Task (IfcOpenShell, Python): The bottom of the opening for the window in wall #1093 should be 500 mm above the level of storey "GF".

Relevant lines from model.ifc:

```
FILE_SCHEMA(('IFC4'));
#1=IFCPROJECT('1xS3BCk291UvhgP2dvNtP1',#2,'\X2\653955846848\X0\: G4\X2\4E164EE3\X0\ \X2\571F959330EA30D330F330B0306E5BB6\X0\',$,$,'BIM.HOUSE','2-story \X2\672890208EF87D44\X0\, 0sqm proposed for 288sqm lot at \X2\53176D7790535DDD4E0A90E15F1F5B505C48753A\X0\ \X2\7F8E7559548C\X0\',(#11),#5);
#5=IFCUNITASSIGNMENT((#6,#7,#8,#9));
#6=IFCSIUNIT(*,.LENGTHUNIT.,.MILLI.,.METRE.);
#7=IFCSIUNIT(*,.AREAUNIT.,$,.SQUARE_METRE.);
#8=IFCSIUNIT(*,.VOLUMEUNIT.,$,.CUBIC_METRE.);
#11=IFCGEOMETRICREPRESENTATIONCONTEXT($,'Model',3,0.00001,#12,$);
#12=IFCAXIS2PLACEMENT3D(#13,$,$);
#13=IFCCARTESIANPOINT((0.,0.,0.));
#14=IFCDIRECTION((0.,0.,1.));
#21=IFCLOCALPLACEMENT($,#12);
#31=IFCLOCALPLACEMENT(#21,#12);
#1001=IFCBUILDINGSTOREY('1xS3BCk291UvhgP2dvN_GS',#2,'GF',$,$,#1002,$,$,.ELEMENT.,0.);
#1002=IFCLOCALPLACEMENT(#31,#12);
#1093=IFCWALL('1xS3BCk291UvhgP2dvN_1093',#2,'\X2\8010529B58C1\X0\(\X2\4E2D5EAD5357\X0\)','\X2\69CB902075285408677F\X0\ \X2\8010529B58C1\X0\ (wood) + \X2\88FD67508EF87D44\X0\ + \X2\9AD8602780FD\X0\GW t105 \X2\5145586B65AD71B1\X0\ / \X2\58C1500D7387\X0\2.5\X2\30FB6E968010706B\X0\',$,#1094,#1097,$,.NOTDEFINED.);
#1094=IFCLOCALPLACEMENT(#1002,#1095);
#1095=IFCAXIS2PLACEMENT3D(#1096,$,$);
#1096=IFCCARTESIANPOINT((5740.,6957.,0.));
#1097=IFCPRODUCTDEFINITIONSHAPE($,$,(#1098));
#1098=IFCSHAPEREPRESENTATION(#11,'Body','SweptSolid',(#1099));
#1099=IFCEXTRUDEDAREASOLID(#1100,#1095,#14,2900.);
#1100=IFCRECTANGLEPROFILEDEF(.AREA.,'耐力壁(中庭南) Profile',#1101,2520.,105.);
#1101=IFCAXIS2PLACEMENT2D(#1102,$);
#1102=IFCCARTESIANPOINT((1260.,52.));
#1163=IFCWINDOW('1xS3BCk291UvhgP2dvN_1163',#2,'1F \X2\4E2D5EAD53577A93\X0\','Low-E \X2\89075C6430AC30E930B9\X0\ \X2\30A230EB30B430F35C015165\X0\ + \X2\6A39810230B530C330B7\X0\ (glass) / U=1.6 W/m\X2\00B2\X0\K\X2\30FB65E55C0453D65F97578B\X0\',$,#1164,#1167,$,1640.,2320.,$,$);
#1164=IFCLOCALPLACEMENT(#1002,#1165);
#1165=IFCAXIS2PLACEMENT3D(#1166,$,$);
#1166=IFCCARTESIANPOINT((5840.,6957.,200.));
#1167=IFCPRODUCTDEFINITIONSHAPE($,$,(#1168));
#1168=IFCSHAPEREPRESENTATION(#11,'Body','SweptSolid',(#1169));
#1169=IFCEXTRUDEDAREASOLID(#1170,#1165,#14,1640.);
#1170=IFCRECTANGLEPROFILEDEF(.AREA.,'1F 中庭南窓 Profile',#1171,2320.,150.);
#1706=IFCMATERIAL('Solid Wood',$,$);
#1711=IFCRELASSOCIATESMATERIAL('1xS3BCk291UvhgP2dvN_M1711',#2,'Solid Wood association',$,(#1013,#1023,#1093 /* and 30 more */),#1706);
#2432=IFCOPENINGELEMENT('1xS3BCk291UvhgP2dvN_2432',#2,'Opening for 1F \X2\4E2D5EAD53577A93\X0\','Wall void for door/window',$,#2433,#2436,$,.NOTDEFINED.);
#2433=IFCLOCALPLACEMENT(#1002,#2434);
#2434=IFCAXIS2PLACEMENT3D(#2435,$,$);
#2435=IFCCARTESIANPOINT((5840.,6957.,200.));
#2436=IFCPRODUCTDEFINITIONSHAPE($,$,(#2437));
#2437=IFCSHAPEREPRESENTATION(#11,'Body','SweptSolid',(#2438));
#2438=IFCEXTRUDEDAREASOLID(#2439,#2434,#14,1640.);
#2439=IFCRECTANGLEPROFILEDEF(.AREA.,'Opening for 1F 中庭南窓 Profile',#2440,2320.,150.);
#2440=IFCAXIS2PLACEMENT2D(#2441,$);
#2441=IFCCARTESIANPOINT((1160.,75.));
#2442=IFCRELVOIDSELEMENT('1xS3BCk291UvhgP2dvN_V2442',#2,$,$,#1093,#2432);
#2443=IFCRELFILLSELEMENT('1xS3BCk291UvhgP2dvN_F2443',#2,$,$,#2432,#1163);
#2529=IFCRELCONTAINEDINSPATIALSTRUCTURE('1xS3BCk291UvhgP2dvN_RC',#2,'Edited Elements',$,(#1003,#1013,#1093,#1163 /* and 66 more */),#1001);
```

```python
import numpy as np
import ifcopenshell
import ifcopenshell.api.geometry
import ifcopenshell.geom
import ifcopenshell.util.element
import ifcopenshell.util.placement
import ifcopenshell.util.shape
import ifcopenshell.util.unit

model = ifcopenshell.open("model.ifc")
unit_scale = ifcopenshell.util.unit.calculate_unit_scale(model)

window = model.by_id(1163)
opening = window.FillsVoids[0].RelatingOpeningElement
storey = ifcopenshell.util.element.get_container(window, ifc_class="IfcBuildingStorey")
level = ifcopenshell.util.placement.get_local_placement(storey.ObjectPlacement)[2, 3]

# The opening's origin need not be at the sill, so measure its lowest point.
shape = ifcopenshell.geom.create_shape(ifcopenshell.geom.settings(), opening)
bottom = ifcopenshell.util.shape.get_shape_bottom_elevation(shape, shape.geometry) / unit_scale
dz = level + 0.5 / unit_scale - bottom

shift = np.array([0.0, 0.0, dz])
# The window is not placed relative to its opening, so move both.
for product in (opening, window):
    matrix = ifcopenshell.util.placement.get_local_placement(product.ObjectPlacement)
    matrix[:3, 3] += shift
    ifcopenshell.api.geometry.edit_object_placement(model, product=product, matrix=matrix, is_si=False)

print(f"moved by {dz * unit_scale:+.3f} m")

model.write("model_rev.ifc")
```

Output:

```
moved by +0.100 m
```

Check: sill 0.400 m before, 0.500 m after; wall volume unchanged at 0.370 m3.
